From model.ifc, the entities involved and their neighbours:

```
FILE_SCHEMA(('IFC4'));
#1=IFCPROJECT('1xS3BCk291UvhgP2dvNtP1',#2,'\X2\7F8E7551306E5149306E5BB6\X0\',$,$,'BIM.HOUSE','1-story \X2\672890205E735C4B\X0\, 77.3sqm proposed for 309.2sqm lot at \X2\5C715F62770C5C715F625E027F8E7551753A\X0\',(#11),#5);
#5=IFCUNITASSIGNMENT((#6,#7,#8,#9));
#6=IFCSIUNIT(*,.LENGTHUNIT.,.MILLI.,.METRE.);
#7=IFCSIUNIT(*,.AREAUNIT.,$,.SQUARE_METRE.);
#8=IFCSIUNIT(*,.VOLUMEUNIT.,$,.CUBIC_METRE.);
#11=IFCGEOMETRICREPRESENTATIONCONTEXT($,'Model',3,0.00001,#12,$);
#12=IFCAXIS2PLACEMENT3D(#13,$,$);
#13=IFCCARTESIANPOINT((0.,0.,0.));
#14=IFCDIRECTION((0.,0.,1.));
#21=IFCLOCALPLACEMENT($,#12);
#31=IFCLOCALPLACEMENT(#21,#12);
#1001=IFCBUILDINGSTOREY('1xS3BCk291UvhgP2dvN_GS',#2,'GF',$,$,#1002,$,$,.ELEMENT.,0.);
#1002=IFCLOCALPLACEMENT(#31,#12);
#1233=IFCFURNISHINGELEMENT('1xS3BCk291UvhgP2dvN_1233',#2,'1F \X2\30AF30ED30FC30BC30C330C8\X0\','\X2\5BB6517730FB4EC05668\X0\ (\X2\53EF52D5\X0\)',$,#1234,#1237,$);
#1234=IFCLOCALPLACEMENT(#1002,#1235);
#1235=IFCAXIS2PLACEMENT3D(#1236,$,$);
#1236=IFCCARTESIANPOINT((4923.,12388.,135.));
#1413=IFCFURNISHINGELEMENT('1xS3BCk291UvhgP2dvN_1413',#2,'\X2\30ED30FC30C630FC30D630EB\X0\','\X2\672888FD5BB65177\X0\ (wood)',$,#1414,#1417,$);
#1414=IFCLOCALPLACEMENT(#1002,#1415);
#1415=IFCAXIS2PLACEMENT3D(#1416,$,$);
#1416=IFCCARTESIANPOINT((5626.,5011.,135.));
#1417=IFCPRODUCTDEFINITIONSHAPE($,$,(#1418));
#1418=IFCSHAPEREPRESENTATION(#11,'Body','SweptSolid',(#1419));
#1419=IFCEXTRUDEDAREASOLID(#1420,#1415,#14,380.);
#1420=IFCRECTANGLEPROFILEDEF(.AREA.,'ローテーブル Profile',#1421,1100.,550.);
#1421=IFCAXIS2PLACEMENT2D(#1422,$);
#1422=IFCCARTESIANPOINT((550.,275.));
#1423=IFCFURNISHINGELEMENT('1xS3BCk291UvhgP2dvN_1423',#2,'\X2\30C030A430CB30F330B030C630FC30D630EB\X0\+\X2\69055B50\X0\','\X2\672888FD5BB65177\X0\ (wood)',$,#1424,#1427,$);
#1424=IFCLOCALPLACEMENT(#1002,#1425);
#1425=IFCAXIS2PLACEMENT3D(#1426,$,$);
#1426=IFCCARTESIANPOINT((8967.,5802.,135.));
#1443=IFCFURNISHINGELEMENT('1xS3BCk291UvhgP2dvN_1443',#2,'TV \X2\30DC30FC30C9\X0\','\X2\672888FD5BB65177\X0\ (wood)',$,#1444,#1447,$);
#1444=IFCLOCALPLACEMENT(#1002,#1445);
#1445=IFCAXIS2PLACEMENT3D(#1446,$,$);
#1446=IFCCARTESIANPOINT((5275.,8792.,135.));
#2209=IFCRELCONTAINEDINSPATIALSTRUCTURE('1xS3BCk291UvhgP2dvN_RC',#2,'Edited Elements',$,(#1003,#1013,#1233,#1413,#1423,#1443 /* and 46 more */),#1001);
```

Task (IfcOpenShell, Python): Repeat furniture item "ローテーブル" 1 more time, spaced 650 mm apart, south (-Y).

```python
import numpy as np
import ifcopenshell
import ifcopenshell.api.geometry
import ifcopenshell.api.root
import ifcopenshell.util.element
import ifcopenshell.util.placement

model = ifcopenshell.open("model.ifc")


def reuse_history(source, copy):
    """copy_class also copies each property set's owner history, people and application; keep the originals."""
    for rel in copy.IsDefinedBy:
        if rel.is_a("IfcRelDefinesByProperties") and (history := rel.RelatingPropertyDefinition.OwnerHistory):
            rel.RelatingPropertyDefinition.OwnerHistory = source.OwnerHistory
            ifcopenshell.util.element.remove_deep2(model, history)


source = model.by_guid("1xS3BCk291UvhgP2dvN_1413")
base = ifcopenshell.util.placement.get_local_placement(source.ObjectPlacement)
step = np.array([0.0, -1.0, 0.0]) * 650.0

for i in range(1, 2):
    copy = ifcopenshell.api.root.copy_class(model, product=source)
    copy.Representation = ifcopenshell.util.element.copy_deep(
        model, source.Representation, exclude=["IfcGeometricRepresentationContext", "IfcRepresentationMap"]
    )
    reuse_history(source, copy)
    matrix = base.copy()
    matrix[:3, 3] += i * step
    print("added at", matrix[:3, 3].round(3) + 0.0)
    ifcopenshell.api.geometry.edit_object_placement(model, product=copy, matrix=matrix, is_si=False)

model.write("model_rev.ifc")
```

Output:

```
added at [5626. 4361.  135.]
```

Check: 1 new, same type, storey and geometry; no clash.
